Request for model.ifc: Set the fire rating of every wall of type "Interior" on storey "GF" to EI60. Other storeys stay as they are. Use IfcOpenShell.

First a look at what the model holds.

```python
import ifcopenshell
import ifcopenshell.util.element

model = ifcopenshell.open("model.ifc")
print(model.schema)
storey = next(s for s in model.by_type("IfcBuildingStorey") if s.Name == "GF")
walls = [e for e in ifcopenshell.util.element.get_decomposition(storey) if e.is_a("IfcWall")]
seen = {}
for e in walls:
    element_type = ifcopenshell.util.element.get_type(e)
    key = (element_type.Name if element_type != e and element_type else None, ifcopenshell.util.element.get_pset(e, "Pset_WallCommon", "FireRating"))
    seen[key] = seen.get(key, 0) + 1
for (name, value), count in sorted(seen.items(), key=str):
    print(count, "x", name, "|", value)
```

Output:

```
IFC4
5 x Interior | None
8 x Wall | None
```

```python
import ifcopenshell
import ifcopenshell.api.pset
import ifcopenshell.util.element

model = ifcopenshell.open("model.ifc")

storey = next(s for s in model.by_type("IfcBuildingStorey") if s.Name == "GF")
walls = [e for e in ifcopenshell.util.element.get_decomposition(storey) if e.is_a("IfcWall")]

count = 0
for e in walls:
    element_type = ifcopenshell.util.element.get_type(e)
    if element_type in (None, e) or element_type.Name != "Interior":
        continue
    # add_pset returns the element's existing set when there is one.
    pset = ifcopenshell.api.pset.add_pset(model, product=e, name="Pset_WallCommon")
    ifcopenshell.api.pset.edit_pset(model, pset=pset, properties={"FireRating": "EI60"})
    count += 1

print(count, "walls updated")

model.write("model_v2.ifc")
```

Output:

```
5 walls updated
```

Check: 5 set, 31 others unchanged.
